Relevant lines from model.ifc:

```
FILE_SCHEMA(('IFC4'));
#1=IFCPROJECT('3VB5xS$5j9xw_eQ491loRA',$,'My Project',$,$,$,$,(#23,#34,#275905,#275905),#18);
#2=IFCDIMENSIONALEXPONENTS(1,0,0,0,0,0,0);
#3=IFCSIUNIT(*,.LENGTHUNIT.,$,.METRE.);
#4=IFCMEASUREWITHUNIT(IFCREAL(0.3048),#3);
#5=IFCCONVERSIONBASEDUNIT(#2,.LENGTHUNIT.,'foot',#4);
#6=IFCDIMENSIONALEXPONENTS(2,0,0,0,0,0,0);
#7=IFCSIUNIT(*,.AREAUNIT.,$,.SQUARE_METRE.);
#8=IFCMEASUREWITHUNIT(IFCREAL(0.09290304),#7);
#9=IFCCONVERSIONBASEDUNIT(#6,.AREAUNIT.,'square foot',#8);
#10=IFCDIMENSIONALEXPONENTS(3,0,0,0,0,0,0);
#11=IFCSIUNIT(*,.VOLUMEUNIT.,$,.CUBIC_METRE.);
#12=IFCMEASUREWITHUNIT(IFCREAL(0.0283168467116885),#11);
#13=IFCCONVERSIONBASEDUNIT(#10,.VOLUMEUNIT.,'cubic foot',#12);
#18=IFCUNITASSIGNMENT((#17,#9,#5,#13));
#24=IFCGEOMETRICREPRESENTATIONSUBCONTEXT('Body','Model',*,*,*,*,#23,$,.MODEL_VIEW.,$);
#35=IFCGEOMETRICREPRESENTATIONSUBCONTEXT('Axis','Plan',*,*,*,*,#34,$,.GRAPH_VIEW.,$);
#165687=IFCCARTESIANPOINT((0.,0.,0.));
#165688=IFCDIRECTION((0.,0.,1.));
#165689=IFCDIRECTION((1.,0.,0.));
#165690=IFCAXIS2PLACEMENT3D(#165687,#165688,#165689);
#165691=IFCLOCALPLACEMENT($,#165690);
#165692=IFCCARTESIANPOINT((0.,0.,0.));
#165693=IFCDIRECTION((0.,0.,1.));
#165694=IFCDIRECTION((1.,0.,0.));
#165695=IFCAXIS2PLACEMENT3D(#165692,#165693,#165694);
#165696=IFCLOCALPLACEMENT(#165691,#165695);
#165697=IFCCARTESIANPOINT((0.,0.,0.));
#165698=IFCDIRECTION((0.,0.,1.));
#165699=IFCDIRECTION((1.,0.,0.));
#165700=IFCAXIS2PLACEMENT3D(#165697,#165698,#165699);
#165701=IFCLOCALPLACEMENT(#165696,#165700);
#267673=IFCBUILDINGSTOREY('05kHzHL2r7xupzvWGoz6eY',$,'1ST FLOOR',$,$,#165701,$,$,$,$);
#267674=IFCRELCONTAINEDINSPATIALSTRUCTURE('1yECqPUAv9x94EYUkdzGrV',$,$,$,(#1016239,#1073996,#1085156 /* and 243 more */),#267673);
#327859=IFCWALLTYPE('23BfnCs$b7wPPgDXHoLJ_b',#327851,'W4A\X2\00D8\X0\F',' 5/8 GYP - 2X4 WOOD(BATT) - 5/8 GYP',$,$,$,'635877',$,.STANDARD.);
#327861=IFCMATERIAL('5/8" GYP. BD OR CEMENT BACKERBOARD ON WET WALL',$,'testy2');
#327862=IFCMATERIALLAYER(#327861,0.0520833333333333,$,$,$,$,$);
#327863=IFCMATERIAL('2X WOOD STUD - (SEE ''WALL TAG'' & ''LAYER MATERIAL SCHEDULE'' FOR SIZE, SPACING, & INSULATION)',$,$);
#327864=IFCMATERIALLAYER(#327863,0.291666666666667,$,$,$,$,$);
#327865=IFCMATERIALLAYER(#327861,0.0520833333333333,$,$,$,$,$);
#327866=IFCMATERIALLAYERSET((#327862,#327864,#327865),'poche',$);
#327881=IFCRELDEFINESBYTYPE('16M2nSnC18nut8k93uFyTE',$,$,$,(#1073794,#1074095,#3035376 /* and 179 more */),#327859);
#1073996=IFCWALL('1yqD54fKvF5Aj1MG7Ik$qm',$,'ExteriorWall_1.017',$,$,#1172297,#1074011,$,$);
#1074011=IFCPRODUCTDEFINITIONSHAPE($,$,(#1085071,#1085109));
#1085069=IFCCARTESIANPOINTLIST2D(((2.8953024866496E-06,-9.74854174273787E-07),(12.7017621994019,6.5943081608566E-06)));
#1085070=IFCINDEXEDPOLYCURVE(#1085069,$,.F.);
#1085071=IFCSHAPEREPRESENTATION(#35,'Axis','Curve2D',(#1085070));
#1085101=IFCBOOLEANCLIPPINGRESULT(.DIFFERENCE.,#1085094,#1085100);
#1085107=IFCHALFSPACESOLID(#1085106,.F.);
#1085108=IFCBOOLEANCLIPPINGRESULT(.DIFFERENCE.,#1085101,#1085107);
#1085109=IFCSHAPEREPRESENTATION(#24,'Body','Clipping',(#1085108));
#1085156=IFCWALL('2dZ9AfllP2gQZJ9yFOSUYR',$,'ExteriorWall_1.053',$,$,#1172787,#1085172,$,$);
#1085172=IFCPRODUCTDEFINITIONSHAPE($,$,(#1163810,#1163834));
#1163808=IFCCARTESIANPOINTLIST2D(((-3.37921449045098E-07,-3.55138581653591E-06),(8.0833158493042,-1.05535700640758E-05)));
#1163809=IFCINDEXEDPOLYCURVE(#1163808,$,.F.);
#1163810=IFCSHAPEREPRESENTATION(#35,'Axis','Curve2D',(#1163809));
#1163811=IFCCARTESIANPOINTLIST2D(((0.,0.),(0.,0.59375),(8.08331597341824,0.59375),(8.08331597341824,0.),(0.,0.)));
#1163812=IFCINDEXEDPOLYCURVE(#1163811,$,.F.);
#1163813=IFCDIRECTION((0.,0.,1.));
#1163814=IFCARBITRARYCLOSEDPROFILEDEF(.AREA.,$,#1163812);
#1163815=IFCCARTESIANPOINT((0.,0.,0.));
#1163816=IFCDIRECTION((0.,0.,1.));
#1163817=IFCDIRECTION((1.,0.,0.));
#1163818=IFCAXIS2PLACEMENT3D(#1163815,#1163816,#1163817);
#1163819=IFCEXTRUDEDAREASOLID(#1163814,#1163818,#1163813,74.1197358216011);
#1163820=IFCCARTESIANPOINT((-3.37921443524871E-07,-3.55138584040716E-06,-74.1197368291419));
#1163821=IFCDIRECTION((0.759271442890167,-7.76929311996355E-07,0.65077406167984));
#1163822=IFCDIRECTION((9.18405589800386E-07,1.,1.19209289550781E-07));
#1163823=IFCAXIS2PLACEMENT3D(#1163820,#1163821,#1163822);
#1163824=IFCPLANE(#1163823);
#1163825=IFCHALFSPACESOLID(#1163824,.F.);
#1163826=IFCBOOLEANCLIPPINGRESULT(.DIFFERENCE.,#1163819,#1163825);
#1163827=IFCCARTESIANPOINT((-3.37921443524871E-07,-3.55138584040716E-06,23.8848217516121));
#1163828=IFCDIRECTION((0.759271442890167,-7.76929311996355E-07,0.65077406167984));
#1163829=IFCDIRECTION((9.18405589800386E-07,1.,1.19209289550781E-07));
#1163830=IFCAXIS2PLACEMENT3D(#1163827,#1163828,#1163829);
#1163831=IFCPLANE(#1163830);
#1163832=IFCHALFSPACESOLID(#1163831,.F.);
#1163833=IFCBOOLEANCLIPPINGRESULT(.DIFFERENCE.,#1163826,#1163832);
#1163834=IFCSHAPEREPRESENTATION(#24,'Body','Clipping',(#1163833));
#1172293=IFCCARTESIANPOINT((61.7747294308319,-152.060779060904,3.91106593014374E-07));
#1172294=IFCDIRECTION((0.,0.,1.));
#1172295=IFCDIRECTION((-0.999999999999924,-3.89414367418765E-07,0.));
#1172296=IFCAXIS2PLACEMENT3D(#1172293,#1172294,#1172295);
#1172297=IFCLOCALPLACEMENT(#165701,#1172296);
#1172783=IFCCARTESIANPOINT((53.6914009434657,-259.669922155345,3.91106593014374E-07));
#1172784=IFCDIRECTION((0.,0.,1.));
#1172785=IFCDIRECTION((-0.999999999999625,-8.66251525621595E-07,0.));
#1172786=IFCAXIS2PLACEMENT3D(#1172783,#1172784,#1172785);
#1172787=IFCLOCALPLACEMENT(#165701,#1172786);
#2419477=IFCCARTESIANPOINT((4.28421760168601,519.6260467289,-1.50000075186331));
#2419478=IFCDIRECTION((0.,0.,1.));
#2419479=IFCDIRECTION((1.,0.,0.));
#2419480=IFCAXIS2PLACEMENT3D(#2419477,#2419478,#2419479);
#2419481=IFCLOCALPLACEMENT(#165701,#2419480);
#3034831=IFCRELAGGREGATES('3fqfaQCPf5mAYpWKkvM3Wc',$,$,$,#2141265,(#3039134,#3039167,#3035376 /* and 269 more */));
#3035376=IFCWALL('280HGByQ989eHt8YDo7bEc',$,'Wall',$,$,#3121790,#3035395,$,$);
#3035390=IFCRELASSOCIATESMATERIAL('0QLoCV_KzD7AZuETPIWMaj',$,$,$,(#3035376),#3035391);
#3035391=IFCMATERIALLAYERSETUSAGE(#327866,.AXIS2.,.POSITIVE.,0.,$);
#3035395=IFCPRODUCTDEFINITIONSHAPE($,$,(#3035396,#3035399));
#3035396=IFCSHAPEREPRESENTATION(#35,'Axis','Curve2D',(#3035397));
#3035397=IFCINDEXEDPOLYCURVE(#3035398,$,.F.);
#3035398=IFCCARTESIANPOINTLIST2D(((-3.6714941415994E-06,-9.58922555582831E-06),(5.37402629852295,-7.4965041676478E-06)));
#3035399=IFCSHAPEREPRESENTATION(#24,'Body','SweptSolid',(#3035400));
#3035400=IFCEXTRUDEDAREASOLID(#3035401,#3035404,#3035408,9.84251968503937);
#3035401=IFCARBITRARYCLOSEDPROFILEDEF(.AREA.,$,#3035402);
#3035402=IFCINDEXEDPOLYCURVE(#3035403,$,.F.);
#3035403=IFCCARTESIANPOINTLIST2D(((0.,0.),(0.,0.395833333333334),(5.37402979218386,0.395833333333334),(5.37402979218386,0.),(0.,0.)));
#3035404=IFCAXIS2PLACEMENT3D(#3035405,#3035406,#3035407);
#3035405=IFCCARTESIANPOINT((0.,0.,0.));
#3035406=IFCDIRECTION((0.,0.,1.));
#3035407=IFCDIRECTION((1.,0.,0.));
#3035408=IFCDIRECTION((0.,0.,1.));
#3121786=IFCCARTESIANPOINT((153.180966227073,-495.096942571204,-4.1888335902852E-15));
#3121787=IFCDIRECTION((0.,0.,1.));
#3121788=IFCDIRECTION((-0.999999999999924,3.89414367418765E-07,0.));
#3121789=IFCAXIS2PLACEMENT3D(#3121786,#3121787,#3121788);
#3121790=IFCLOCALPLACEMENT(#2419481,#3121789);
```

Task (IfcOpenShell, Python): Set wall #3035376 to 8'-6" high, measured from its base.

```python
import ifcopenshell
import ifcopenshell.geom
import ifcopenshell.util.representation
import ifcopenshell.util.shape
import ifcopenshell.util.unit

model = ifcopenshell.open("model.ifc")
unit_scale = ifcopenshell.util.unit.calculate_unit_scale(model)
settings = ifcopenshell.geom.settings()


def volume(element):
    """Net volume in cubic metres, openings subtracted."""
    shape = ifcopenshell.geom.create_shape(settings, element)
    return ifcopenshell.util.shape.get_volume(shape.geometry)


wall = model.by_guid("280HGByQ989eHt8YDo7bEc")
before = volume(wall)

body = ifcopenshell.util.representation.get_representation(wall, "Model", "Body")
solid = body.Items[0]
old_height = solid.Depth
solid.Depth = 102 * 0.0254 / unit_scale
after = volume(wall)

print(f"height {old_height:g} -> {solid.Depth:g}, volume {before:.3f} -> {after:.3f} m3")

model.write("model_rev.ifc")
```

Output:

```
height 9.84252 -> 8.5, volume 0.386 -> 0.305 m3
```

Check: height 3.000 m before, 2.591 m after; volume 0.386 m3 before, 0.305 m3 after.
